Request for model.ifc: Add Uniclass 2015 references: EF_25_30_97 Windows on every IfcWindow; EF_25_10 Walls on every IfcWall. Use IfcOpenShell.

First a look at what the model holds.

```python
import ifcopenshell

model = ifcopenshell.open("model.ifc")
print(model.schema)
print("classifications:", [c.Name for c in model.by_type("IfcClassification")])
for ifc_class in ("IfcDoor", "IfcRoof", "IfcStair", "IfcWall", "IfcWindow"):
    print(ifc_class, len(model.by_type(ifc_class)))
```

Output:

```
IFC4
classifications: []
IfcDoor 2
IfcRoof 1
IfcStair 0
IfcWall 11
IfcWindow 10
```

```python
import ifcopenshell
import ifcopenshell.api.classification

model = ifcopenshell.open("model.ifc")

system = ifcopenshell.api.classification.add_classification(model, classification="Uniclass 2015")

codes = {
    "IfcWindow": ("EF_25_30_97", "Windows"),
    "IfcWall": ("EF_25_10", "Walls"),
}
for ifc_class, (code, name) in codes.items():
    products = model.by_type(ifc_class)
    ifcopenshell.api.classification.add_reference(
        model, products=products, classification=system, identification=code, name=name
    )
    print(code, len(products))

model.write("model_edited.ifc")
```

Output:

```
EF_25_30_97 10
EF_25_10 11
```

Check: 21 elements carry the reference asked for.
